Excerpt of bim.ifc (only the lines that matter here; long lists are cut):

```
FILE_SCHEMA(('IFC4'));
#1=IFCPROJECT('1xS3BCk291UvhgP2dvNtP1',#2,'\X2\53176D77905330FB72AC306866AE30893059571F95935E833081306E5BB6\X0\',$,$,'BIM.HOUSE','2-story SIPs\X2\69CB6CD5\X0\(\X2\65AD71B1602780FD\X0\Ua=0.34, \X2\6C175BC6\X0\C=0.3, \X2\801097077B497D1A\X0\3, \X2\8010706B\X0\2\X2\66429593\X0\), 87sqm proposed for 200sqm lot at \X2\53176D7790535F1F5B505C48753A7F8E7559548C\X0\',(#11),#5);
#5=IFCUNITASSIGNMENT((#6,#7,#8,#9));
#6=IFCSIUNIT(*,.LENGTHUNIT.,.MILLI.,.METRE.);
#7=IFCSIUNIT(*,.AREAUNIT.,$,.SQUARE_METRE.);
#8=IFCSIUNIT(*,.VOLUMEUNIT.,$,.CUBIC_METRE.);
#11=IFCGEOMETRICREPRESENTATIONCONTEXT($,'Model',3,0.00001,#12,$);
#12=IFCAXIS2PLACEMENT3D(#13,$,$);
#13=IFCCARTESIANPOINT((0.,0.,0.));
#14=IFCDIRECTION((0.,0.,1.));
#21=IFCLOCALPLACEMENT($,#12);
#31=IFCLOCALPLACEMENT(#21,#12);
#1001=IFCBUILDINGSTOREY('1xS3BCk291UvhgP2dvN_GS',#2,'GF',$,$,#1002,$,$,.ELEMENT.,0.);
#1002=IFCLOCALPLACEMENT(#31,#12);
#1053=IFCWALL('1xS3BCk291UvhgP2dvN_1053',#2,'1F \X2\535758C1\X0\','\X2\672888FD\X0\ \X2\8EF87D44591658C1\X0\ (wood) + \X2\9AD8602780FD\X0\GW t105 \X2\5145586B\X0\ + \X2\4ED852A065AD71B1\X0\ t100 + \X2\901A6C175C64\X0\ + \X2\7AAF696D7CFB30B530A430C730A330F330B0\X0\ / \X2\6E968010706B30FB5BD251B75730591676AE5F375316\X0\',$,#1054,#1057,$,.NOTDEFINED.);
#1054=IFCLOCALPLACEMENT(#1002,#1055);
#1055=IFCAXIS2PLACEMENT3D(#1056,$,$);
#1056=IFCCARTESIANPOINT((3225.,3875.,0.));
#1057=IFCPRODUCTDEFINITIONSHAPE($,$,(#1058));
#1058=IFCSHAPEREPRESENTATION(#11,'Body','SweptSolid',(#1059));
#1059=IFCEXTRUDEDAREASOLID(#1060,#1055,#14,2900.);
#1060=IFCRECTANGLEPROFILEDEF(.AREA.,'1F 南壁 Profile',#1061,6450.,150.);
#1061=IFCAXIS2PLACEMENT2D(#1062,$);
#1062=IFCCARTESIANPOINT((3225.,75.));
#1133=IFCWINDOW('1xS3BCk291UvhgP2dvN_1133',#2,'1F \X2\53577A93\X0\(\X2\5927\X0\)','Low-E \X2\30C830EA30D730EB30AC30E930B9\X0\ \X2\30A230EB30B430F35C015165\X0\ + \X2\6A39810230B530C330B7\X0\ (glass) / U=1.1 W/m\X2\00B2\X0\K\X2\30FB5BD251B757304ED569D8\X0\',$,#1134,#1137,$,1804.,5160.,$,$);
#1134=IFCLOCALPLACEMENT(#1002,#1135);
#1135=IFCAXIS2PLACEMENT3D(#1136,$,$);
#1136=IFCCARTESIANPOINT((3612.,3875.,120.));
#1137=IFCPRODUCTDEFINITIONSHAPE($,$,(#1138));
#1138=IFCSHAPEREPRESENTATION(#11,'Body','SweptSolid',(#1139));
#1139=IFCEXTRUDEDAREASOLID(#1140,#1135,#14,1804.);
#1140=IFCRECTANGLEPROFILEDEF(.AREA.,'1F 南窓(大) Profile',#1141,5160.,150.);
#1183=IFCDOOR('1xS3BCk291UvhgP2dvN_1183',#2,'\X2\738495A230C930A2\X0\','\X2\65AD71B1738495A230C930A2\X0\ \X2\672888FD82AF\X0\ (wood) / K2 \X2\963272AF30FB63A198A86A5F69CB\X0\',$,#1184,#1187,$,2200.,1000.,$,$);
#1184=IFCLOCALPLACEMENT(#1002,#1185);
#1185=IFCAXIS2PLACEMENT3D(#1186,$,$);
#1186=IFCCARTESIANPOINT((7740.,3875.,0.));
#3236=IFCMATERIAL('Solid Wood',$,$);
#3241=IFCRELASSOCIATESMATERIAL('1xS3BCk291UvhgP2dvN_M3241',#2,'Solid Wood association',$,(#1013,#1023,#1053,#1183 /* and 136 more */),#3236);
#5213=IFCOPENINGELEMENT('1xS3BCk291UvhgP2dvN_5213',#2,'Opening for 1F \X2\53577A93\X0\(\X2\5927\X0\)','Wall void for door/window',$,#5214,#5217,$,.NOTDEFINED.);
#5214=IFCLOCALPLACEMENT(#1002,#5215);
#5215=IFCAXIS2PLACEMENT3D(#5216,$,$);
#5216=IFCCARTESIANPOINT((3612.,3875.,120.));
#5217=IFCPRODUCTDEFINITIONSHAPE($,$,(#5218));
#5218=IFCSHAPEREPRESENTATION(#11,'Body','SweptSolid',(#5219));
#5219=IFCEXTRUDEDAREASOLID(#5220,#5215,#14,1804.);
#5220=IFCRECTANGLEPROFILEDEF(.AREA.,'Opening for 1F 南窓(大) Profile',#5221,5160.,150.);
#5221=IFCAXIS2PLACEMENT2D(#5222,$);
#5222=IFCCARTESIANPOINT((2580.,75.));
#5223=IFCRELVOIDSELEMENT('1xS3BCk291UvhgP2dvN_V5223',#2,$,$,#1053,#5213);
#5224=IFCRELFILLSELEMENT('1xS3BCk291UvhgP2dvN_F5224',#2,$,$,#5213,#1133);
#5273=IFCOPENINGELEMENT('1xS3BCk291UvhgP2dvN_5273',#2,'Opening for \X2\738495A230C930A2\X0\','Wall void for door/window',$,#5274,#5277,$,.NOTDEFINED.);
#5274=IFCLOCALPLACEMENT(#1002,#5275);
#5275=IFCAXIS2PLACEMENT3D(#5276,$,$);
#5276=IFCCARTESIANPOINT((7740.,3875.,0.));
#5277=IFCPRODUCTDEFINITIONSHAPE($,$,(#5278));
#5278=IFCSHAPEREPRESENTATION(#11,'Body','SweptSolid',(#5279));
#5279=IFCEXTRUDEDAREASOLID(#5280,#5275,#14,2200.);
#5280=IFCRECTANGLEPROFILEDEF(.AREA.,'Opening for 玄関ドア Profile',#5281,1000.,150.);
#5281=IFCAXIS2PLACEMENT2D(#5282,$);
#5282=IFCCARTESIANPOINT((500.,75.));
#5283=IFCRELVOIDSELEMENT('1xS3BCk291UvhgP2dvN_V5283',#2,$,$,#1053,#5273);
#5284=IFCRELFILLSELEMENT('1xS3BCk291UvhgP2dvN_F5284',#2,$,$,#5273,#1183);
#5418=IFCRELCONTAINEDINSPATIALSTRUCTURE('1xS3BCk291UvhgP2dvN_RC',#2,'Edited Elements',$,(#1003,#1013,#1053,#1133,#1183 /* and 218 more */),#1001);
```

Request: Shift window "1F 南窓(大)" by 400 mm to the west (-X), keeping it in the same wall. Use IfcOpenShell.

```python
import ifcopenshell
import ifcopenshell.api.geometry
import ifcopenshell.util.placement

model = ifcopenshell.open("bim.ifc")

window = model.by_guid("1xS3BCk291UvhgP2dvN_1133")
opening = window.FillsVoids[0].RelatingOpeningElement
wall = opening.VoidsElements[0].RelatingBuildingElement

wall_matrix = ifcopenshell.util.placement.get_local_placement(wall.ObjectPlacement)
shift = wall_matrix[:3, 0] * -400.0
before = ifcopenshell.util.placement.get_local_placement(window.ObjectPlacement)[:3, 3].copy()

# The window is not placed relative to its opening, so move both.
for product in (opening, window):
    matrix = ifcopenshell.util.placement.get_local_placement(product.ObjectPlacement)
    matrix[:3, 3] += shift
    ifcopenshell.api.geometry.edit_object_placement(model, product=product, matrix=matrix, is_si=False)

after = ifcopenshell.util.placement.get_local_placement(window.ObjectPlacement)[:3, 3]
print("window moved by", (after - before).round(3) + 0.0)

model.write("bim_updated.ifc")
```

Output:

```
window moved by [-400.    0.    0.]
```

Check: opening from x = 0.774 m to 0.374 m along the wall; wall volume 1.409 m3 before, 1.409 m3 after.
